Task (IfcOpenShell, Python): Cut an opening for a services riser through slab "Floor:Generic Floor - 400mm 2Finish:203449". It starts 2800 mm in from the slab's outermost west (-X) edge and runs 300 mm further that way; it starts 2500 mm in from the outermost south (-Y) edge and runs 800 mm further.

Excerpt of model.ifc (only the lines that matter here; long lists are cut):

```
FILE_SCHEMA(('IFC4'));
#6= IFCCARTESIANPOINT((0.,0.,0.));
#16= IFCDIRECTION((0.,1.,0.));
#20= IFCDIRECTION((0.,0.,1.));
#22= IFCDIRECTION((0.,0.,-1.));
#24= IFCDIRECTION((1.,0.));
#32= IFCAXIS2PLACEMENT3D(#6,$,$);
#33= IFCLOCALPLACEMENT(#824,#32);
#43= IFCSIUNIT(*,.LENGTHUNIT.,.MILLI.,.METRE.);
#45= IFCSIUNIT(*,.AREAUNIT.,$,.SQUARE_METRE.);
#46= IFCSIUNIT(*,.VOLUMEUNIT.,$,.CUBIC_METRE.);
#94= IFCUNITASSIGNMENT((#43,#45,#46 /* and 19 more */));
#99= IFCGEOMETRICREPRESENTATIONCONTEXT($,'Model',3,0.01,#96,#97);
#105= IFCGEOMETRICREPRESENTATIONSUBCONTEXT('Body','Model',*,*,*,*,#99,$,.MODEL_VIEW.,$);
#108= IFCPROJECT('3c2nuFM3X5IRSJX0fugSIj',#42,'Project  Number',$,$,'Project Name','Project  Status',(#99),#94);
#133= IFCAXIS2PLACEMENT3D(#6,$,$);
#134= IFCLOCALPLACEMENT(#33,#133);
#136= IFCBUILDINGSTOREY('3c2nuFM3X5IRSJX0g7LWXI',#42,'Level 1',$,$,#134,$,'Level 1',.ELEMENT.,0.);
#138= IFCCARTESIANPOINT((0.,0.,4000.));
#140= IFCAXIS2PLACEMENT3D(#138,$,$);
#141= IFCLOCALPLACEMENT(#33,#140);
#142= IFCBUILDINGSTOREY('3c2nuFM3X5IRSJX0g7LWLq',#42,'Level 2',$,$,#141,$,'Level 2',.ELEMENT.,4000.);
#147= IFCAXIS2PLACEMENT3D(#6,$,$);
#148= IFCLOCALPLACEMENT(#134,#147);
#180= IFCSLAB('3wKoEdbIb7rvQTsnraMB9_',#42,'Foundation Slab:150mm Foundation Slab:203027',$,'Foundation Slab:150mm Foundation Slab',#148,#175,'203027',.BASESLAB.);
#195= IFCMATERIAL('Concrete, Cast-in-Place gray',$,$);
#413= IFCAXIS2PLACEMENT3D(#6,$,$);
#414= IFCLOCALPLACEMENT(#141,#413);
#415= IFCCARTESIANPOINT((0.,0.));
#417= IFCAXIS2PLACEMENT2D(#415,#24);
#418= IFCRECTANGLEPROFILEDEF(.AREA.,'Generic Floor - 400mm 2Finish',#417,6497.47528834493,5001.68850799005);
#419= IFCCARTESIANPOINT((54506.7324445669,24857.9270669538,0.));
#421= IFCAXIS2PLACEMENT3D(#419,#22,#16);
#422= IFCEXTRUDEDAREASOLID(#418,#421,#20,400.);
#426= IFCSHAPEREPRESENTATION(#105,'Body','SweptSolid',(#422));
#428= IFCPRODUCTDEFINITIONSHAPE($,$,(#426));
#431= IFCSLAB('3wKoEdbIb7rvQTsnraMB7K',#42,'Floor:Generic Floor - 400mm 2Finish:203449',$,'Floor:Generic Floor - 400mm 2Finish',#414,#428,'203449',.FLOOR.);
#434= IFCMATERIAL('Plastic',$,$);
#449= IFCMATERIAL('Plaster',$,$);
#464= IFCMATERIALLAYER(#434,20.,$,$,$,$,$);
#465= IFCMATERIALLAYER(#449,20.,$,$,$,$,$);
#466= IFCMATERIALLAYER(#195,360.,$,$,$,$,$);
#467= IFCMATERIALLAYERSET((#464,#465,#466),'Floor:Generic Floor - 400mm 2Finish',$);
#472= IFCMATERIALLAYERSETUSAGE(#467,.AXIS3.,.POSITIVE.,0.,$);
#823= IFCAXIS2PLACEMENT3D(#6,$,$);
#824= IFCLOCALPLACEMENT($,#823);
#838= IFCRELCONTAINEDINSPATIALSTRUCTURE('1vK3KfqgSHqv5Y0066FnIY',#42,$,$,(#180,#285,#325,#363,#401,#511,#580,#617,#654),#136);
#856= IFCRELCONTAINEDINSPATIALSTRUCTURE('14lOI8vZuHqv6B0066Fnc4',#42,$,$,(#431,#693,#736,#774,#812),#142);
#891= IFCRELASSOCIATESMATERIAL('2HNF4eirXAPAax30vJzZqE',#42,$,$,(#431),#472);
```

```python
import numpy as np
import ifcopenshell
import ifcopenshell.api.feature
import ifcopenshell.api.geometry
import ifcopenshell.api.root
import ifcopenshell.geom
import ifcopenshell.util.placement
import ifcopenshell.util.representation
import ifcopenshell.util.shape
import ifcopenshell.util.unit

model = ifcopenshell.open("model.ifc")
unit_scale = ifcopenshell.util.unit.calculate_unit_scale(model)
settings = ifcopenshell.geom.settings()


def volume(element):
    """Net volume in cubic metres, openings subtracted."""
    shape = ifcopenshell.geom.create_shape(settings, element)
    return ifcopenshell.util.shape.get_volume(shape.geometry)


slab = model.by_guid("3wKoEdbIb7rvQTsnraMB7K")
before = volume(slab)

# Extent in the slab's own axes, in metres. The edges named are its -X and -Y sides.
slab_shape = ifcopenshell.geom.create_shape(settings, slab)
vertices = ifcopenshell.util.shape.get_vertices(slab_shape.geometry)
x_min, y_min, bottom = vertices.min(axis=0)
top = vertices[:, 2].max()

opening = ifcopenshell.api.root.create_entity(model, ifc_class="IfcOpeningElement", name="Services riser opening", predefined_type="OPENING")
context = ifcopenshell.util.representation.get_context(model, "Model", "Body", "MODEL_VIEW")
width, depth = 0.3, 0.8
outline = [(0.0, 0.0), (width, 0.0), (width, depth), (0.0, depth), (0.0, 0.0)]
# Overshoot both faces by 50 mm so the cut is clean.
shape = ifcopenshell.api.geometry.add_slab_representation(
    model, context=context, depth=top - bottom + 0.1, polyline=outline
)
ifcopenshell.api.geometry.assign_representation(model, product=opening, representation=shape)

matrix = ifcopenshell.util.placement.get_local_placement(slab.ObjectPlacement)
matrix[:, 3] = matrix @ np.append(np.array([x_min + 2.8, y_min + 2.5, bottom - 0.05]) / unit_scale, 1.0)
ifcopenshell.api.geometry.edit_object_placement(model, product=opening, matrix=matrix, is_si=False)
ifcopenshell.api.feature.add_feature(model, feature=opening, element=slab)

after = volume(slab)

print(f"slab volume {before:.3f} -> {after:.3f} m3")

model.write("model_edited.ifc")
```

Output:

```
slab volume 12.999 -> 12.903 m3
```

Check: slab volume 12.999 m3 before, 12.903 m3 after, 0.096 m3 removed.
